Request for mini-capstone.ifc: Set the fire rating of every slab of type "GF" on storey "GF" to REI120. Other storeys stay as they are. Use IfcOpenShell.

First a look at what the model holds.

```python
import ifcopenshell
import ifcopenshell.util.element

model = ifcopenshell.open("mini-capstone.ifc")
print(model.schema)
storey = next(s for s in model.by_type("IfcBuildingStorey") if s.Name == "GF")
slabs = [e for e in ifcopenshell.util.element.get_decomposition(storey) if e.is_a("IfcSlab")]
seen = {}
for e in slabs:
    element_type = ifcopenshell.util.element.get_type(e)
    key = (element_type.Name if element_type != e and element_type else None, ifcopenshell.util.element.get_pset(e, "Pset_SlabCommon", "FireRating"))
    seen[key] = seen.get(key, 0) + 1
for (name, value), count in sorted(seen.items(), key=str):
    print(count, "x", name, "|", value)
```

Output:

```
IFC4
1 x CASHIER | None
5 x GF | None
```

```python
import ifcopenshell
import ifcopenshell.api.pset
import ifcopenshell.util.element

model = ifcopenshell.open("mini-capstone.ifc")

storey = next(s for s in model.by_type("IfcBuildingStorey") if s.Name == "GF")
slabs = [e for e in ifcopenshell.util.element.get_decomposition(storey) if e.is_a("IfcSlab")]

count = 0
for e in slabs:
    element_type = ifcopenshell.util.element.get_type(e)
    if element_type in (None, e) or element_type.Name != "GF":
        continue
    # add_pset returns the element's existing set when there is one.
    pset = ifcopenshell.api.pset.add_pset(model, product=e, name="Pset_SlabCommon")
    ifcopenshell.api.pset.edit_pset(model, pset=pset, properties={"FireRating": "REI120"})
    count += 1

print(count, "slabs updated")

model.write("mini-capstone-out.ifc")
```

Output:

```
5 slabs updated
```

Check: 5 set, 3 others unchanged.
